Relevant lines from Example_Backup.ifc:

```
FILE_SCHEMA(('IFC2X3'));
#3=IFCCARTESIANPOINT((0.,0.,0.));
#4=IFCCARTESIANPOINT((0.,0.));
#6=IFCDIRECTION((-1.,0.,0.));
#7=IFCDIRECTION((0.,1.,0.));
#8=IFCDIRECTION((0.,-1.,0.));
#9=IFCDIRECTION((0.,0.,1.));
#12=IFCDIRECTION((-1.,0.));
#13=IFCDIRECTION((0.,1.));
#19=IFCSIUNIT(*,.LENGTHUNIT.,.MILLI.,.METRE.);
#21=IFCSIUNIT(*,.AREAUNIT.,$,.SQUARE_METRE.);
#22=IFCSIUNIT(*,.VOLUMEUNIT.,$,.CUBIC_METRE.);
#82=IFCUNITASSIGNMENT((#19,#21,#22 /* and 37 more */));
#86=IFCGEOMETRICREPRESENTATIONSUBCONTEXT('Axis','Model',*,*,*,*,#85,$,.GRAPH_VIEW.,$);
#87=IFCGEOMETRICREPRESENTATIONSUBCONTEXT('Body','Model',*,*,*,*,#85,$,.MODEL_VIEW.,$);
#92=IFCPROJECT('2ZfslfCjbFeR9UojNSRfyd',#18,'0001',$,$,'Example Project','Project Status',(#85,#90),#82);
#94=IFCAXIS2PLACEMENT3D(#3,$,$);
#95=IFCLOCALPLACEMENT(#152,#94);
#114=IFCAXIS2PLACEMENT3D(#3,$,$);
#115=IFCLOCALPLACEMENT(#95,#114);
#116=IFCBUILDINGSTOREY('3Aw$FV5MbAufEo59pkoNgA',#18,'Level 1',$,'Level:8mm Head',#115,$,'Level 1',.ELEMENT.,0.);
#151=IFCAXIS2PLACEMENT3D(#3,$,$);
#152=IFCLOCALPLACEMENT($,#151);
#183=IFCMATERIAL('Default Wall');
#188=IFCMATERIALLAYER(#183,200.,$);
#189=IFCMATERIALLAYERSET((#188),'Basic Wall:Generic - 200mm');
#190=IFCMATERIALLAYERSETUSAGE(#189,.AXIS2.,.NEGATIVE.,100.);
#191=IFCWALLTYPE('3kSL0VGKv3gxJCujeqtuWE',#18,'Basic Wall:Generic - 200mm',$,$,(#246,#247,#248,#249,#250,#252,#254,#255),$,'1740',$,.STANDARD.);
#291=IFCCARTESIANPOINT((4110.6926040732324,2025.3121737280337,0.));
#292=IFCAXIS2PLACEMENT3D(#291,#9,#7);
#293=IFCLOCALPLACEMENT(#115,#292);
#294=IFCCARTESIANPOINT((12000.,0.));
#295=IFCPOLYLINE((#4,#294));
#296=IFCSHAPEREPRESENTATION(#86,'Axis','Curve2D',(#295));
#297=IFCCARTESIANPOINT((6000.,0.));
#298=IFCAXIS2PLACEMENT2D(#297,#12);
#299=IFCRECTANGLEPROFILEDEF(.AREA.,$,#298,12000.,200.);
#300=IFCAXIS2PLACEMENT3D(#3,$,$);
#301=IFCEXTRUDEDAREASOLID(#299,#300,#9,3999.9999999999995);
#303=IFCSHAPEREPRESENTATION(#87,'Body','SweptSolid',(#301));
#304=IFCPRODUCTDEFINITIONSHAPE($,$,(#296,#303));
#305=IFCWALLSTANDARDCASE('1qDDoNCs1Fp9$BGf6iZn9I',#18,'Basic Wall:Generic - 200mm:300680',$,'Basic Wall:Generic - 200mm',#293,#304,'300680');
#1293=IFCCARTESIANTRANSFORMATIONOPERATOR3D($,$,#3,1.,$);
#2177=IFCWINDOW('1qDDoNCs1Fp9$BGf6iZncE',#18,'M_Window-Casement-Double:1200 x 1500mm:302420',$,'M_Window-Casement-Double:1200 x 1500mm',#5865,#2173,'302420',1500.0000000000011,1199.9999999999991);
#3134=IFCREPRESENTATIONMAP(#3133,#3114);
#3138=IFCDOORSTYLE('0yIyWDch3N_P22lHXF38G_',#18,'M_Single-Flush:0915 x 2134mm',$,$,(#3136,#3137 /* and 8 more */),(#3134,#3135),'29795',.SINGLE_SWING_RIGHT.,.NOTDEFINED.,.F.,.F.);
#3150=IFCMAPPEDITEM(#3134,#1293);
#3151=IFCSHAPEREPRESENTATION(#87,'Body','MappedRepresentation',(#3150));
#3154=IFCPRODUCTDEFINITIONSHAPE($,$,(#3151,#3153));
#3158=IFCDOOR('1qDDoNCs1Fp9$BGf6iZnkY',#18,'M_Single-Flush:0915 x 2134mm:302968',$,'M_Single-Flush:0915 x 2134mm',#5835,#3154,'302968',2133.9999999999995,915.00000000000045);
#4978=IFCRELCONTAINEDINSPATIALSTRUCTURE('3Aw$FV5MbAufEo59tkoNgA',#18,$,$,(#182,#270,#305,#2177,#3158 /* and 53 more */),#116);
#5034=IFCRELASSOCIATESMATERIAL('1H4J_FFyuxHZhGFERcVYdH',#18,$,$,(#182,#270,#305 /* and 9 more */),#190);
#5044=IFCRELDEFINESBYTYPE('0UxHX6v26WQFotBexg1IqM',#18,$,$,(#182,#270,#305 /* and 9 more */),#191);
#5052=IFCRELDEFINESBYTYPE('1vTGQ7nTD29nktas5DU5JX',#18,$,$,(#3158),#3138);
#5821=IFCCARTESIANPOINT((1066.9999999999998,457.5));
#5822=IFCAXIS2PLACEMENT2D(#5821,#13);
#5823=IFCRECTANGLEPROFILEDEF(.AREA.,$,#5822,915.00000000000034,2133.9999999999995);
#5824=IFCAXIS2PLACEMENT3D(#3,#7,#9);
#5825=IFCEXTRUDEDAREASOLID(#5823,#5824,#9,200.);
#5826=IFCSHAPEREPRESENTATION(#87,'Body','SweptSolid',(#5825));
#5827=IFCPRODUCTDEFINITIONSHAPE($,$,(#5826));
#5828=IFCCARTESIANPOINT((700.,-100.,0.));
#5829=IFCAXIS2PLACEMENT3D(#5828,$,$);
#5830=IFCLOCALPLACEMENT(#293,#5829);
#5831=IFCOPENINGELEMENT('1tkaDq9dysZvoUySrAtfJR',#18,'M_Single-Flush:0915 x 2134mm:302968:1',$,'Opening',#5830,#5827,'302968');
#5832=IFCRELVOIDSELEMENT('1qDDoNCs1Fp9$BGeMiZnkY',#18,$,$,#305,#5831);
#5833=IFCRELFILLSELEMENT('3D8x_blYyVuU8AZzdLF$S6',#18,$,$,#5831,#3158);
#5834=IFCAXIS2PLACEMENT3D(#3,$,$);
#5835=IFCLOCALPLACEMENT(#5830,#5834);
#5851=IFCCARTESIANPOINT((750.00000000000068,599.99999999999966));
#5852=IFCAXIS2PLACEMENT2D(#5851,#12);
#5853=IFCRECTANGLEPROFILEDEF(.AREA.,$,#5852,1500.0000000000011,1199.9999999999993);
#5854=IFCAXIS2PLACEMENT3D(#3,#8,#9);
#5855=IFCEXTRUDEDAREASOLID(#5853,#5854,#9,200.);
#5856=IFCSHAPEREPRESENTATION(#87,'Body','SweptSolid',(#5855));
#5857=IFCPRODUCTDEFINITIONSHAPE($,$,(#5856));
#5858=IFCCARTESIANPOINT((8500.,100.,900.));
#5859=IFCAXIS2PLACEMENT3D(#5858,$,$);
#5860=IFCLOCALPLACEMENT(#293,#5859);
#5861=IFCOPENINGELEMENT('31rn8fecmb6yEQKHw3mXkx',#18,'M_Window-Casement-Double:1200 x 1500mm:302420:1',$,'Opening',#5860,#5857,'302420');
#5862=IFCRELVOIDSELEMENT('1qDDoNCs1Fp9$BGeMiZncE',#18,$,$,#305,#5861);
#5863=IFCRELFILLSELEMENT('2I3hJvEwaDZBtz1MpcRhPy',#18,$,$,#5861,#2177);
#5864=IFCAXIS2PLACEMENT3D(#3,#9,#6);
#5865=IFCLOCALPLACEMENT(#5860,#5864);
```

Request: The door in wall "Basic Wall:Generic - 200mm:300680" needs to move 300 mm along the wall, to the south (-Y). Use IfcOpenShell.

```python
import ifcopenshell
import ifcopenshell.api.geometry
import ifcopenshell.util.placement

model = ifcopenshell.open("Example_Backup.ifc")

door = model.by_guid("1qDDoNCs1Fp9$BGf6iZnkY")
opening = door.FillsVoids[0].RelatingOpeningElement
wall = opening.VoidsElements[0].RelatingBuildingElement

wall_matrix = ifcopenshell.util.placement.get_local_placement(wall.ObjectPlacement)
shift = wall_matrix[:3, 0] * -300.0
before = ifcopenshell.util.placement.get_local_placement(door.ObjectPlacement)[:3, 3].copy()

# The door is placed relative to its opening, so it follows when the opening moves.
matrix = ifcopenshell.util.placement.get_local_placement(opening.ObjectPlacement)
matrix[:3, 3] += shift
ifcopenshell.api.geometry.edit_object_placement(
    model, product=opening, matrix=matrix, is_si=False, should_transform_children=True
)

after = ifcopenshell.util.placement.get_local_placement(door.ObjectPlacement)[:3, 3]
print("door moved by", (after - before).round(3) + 0.0)

model.write("Example_Backup_edited.ifc")
```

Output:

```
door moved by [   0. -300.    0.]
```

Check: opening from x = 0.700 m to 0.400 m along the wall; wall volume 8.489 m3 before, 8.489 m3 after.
